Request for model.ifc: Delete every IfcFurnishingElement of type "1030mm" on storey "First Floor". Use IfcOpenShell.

First a look at what the model holds.

```python
import ifcopenshell
import ifcopenshell.util.element

model = ifcopenshell.open("model.ifc")
print(model.schema)
storey = next(s for s in model.by_type("IfcBuildingStorey") if s.Name == "First Floor")
furniture = [e for e in ifcopenshell.util.element.get_decomposition(storey) if e.is_a("IfcFurnishingElement")]
seen = {}
for e in furniture:
    element_type = ifcopenshell.util.element.get_type(e)
    name = element_type.Name if element_type not in (None, e) else None
    seen[name] = seen.get(name, 0) + 1
for name, count in sorted(seen.items(), key=str):
    print(count, "x", name)
```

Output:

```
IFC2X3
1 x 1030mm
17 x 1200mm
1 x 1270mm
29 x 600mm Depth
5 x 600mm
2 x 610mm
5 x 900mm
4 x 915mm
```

```python
import ifcopenshell
import ifcopenshell.api.root
import ifcopenshell.util.element

model = ifcopenshell.open("model.ifc")

storey = next(s for s in model.by_type("IfcBuildingStorey") if s.Name == "First Floor")
furniture = [e for e in ifcopenshell.util.element.get_decomposition(storey) if e.is_a("IfcFurnishingElement")]
targets = [e for e in furniture if (t := ifcopenshell.util.element.get_type(e)) not in (None, e) and t.Name == "1030mm"]

for e in targets:
    ifcopenshell.api.root.remove_product(model, product=e)
print(len(targets), "removed")

model.write("model_updated.ifc")
```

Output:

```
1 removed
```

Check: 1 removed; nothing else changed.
